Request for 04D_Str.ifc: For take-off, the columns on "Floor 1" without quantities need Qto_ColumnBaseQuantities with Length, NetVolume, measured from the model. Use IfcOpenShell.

First a look at what the model holds.

```python
import ifcopenshell
import ifcopenshell.util.element
import ifcopenshell.util.unit

model = ifcopenshell.open("04D_Str.ifc")
print(model.schema)
for unit_type in ("LENGTHUNIT", "AREAUNIT", "VOLUMEUNIT"):
    print(unit_type, ifcopenshell.util.unit.calculate_unit_scale(model, unit_type))
storey = next(s for s in model.by_type("IfcBuildingStorey") if s.Name == "Floor 1")
columns = [e for e in ifcopenshell.util.element.get_decomposition(storey) if e.is_a("IfcColumn")]
for e in sorted(columns, key=lambda e: e.id()):
    print(e.id(), e.is_a(), e.Name, list(ifcopenshell.util.element.get_psets(e, qtos_only=True)), sep=" | ")
```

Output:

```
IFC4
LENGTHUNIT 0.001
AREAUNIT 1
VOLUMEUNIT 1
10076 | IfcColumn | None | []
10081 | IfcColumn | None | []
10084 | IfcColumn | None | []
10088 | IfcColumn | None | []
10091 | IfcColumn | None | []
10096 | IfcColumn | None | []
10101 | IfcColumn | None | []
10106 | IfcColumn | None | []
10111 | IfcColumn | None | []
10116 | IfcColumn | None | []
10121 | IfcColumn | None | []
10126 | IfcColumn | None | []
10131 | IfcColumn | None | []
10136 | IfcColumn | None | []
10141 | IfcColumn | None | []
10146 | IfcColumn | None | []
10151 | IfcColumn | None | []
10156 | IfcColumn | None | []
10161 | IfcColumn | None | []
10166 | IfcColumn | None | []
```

```python
import ifcopenshell
import ifcopenshell.api.pset
import ifcopenshell.geom
import ifcopenshell.util.element
import ifcopenshell.util.shape
import ifcopenshell.util.unit

model = ifcopenshell.open("04D_Str.ifc")
unit_scale = ifcopenshell.util.unit.calculate_unit_scale(model)
volume_scale = ifcopenshell.util.unit.calculate_unit_scale(model, "VOLUMEUNIT")
settings = ifcopenshell.geom.settings()

storey = next(s for s in model.by_type("IfcBuildingStorey") if s.Name == "Floor 1")
columns = [e for e in ifcopenshell.util.element.get_decomposition(storey) if e.is_a("IfcColumn")]

for e in sorted(columns, key=lambda e: e.id()):
    if ifcopenshell.util.element.get_psets(e, qtos_only=True, should_inherit=False):
        continue
    # Geometry comes back in metres, in the element's own axes.
    shape = ifcopenshell.geom.create_shape(settings, e)
    values = {
        "Length": ifcopenshell.util.shape.get_z(shape.geometry) / unit_scale,
        "NetVolume": ifcopenshell.util.shape.get_volume(shape.geometry) / volume_scale,
    }
    qto = ifcopenshell.api.pset.add_qto(model, product=e, name="Qto_ColumnBaseQuantities")
    ifcopenshell.api.pset.edit_qto(model, qto=qto, properties=values)
    print(e.id(), {k: round(v, 3) for k, v in values.items()})

model.write("04D_Str_rev.ifc")
```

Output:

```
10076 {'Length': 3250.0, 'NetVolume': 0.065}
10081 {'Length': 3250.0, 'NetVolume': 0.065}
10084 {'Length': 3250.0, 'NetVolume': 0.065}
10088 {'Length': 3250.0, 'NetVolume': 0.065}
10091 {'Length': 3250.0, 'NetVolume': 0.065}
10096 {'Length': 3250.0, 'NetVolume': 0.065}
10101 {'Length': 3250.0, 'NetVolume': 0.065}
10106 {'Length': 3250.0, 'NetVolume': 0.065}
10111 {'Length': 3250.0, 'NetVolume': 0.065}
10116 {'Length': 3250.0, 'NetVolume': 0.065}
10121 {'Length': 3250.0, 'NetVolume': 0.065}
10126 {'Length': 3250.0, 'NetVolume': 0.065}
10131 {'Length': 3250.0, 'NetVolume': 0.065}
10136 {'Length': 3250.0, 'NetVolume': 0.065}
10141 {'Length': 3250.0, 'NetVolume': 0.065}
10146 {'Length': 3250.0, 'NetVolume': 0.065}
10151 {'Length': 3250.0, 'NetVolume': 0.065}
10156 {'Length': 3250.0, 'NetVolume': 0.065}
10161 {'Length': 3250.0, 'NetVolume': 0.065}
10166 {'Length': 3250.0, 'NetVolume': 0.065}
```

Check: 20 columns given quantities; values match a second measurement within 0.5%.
